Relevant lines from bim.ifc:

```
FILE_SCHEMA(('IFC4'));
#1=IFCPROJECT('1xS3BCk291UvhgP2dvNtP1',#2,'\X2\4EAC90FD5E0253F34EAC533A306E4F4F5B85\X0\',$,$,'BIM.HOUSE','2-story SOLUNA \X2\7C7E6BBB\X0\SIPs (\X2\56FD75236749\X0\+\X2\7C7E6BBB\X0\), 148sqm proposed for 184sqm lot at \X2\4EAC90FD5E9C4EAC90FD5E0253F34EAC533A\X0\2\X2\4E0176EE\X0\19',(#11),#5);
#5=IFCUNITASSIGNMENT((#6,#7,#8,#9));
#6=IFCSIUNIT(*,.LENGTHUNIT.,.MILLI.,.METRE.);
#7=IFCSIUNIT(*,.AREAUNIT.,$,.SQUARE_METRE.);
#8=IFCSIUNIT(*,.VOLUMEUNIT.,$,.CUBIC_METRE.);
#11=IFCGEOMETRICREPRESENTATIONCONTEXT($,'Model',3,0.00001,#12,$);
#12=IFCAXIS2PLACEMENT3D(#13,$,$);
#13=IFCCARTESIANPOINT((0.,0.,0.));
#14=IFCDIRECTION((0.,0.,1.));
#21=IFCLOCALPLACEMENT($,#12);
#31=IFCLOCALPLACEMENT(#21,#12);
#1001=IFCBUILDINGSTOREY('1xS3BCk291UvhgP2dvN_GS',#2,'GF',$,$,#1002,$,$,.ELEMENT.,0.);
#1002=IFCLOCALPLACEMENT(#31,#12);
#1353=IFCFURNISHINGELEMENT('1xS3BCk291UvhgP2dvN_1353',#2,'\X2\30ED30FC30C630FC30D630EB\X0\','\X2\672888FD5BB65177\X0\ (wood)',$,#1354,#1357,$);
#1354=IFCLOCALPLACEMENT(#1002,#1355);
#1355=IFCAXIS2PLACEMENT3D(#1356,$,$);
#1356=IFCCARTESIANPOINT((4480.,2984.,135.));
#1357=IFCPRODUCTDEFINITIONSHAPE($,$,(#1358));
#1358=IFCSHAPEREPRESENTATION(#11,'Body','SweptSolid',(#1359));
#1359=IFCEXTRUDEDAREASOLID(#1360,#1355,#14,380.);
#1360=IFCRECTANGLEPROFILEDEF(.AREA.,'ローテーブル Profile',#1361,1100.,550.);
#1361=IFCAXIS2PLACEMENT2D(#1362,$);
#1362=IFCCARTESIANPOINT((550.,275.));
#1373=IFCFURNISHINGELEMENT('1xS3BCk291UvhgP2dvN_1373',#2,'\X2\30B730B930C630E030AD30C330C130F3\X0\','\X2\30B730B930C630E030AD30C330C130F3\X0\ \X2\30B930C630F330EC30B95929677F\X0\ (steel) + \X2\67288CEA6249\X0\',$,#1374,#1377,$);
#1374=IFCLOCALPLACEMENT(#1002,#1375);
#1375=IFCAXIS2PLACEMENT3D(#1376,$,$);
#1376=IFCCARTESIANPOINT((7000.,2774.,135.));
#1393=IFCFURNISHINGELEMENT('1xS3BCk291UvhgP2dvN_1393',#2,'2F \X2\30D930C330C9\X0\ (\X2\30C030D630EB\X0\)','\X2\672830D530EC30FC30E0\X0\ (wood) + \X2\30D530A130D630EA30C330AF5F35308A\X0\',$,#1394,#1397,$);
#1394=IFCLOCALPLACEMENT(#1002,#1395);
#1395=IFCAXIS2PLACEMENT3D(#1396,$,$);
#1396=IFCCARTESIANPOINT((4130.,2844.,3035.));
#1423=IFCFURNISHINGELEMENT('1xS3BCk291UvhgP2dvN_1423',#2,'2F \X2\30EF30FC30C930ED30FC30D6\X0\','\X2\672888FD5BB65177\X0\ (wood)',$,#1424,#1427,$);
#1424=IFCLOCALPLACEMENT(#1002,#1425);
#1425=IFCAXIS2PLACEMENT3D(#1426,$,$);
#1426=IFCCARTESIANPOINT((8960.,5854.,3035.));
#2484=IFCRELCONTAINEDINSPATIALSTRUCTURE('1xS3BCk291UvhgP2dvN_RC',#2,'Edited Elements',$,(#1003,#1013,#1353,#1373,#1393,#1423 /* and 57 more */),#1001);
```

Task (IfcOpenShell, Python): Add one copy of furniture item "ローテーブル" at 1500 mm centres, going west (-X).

```python
import numpy as np
import ifcopenshell
import ifcopenshell.api.geometry
import ifcopenshell.api.root
import ifcopenshell.util.element
import ifcopenshell.util.placement

model = ifcopenshell.open("bim.ifc")


def reuse_history(source, copy):
    """copy_class also copies each property set's owner history, people and application; keep the originals."""
    for rel in copy.IsDefinedBy:
        if rel.is_a("IfcRelDefinesByProperties") and (history := rel.RelatingPropertyDefinition.OwnerHistory):
            rel.RelatingPropertyDefinition.OwnerHistory = source.OwnerHistory
            ifcopenshell.util.element.remove_deep2(model, history)


source = model.by_guid("1xS3BCk291UvhgP2dvN_1353")
base = ifcopenshell.util.placement.get_local_placement(source.ObjectPlacement)
step = np.array([-1.0, 0.0, 0.0]) * 1500.0

for i in range(1, 2):
    copy = ifcopenshell.api.root.copy_class(model, product=source)
    copy.Representation = ifcopenshell.util.element.copy_deep(
        model, source.Representation, exclude=["IfcGeometricRepresentationContext", "IfcRepresentationMap"]
    )
    reuse_history(source, copy)
    matrix = base.copy()
    matrix[:3, 3] += i * step
    print("added at", matrix[:3, 3].round(3) + 0.0)
    ifcopenshell.api.geometry.edit_object_placement(model, product=copy, matrix=matrix, is_si=False)

model.write("bim_v2.ifc")
```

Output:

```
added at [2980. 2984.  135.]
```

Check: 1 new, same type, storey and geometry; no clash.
